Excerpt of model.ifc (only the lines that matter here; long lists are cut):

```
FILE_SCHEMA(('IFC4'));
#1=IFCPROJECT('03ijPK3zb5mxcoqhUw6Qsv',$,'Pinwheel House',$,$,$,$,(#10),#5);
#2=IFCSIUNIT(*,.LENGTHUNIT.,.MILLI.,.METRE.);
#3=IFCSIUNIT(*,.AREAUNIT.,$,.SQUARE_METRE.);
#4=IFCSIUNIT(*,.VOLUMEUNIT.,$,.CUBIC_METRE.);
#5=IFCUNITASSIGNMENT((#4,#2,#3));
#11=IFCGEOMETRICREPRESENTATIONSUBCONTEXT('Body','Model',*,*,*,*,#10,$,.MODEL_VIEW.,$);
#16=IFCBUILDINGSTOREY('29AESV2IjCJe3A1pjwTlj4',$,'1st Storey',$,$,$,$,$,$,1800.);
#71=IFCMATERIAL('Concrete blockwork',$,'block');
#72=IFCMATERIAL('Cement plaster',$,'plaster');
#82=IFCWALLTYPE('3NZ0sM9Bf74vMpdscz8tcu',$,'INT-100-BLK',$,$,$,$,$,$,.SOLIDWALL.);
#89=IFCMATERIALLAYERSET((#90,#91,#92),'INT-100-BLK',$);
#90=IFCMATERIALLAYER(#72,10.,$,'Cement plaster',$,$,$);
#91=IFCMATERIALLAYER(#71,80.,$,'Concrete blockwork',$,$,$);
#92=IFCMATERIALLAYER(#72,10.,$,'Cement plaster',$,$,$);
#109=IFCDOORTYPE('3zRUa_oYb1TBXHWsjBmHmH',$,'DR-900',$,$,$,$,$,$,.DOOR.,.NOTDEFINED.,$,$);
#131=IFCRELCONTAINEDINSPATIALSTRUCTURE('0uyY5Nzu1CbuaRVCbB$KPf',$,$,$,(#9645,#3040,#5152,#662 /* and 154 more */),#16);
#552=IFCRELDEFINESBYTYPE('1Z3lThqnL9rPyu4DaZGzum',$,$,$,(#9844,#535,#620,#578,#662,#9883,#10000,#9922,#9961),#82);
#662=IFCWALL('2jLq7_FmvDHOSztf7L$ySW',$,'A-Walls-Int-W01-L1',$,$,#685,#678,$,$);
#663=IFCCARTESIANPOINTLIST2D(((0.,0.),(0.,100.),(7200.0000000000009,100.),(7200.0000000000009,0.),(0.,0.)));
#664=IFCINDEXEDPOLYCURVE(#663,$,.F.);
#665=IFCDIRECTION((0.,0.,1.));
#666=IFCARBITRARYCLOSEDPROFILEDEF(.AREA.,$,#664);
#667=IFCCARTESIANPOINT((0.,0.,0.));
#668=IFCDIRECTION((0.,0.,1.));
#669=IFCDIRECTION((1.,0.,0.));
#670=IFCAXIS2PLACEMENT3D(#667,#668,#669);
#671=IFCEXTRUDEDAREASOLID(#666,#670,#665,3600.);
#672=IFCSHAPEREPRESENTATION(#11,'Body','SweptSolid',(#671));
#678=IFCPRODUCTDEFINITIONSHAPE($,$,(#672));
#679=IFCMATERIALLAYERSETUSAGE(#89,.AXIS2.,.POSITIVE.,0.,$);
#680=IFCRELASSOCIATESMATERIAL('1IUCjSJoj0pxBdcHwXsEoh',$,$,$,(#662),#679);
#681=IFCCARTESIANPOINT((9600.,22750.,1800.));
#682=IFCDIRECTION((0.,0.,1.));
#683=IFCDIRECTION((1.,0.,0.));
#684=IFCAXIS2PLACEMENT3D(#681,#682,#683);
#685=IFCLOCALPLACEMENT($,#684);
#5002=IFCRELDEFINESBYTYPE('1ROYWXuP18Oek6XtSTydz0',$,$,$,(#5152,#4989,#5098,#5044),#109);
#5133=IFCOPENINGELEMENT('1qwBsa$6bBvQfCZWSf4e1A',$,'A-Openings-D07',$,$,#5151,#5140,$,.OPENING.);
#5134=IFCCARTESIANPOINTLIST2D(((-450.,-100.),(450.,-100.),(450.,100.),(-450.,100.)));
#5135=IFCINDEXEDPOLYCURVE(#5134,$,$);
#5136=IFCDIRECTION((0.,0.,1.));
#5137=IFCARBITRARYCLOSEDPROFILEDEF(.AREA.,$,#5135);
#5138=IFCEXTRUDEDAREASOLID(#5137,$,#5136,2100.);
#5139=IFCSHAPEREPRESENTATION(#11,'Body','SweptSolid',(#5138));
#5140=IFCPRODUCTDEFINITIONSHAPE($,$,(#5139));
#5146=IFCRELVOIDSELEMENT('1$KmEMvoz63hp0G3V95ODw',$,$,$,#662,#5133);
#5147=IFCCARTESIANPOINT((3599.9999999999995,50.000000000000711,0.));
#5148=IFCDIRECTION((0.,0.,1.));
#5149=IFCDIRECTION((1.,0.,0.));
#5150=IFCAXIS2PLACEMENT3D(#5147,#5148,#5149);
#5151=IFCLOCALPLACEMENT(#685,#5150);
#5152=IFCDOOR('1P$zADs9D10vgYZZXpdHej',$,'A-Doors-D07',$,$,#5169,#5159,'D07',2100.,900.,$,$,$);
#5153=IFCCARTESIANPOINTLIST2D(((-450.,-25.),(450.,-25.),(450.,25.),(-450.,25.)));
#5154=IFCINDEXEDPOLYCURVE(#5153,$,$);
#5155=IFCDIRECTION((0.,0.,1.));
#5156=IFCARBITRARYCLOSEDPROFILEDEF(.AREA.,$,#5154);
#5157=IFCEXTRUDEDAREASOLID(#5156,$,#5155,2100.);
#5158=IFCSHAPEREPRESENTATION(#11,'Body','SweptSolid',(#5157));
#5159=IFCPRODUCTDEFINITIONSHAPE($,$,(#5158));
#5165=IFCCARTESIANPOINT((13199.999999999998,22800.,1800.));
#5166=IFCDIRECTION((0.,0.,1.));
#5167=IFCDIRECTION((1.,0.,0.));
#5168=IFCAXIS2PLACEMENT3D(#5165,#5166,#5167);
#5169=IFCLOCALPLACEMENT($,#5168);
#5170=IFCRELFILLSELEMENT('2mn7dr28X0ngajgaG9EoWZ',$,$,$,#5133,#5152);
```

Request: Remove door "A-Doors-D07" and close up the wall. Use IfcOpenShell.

```python
import ifcopenshell
import ifcopenshell.api.feature
import ifcopenshell.api.root
import ifcopenshell.geom
import ifcopenshell.util.shape

model = ifcopenshell.open("model.ifc")
settings = ifcopenshell.geom.settings()


def volume(element):
    """Net volume in cubic metres, openings subtracted."""
    shape = ifcopenshell.geom.create_shape(settings, element)
    return ifcopenshell.util.shape.get_volume(shape.geometry)


door = model.by_guid("1P$zADs9D10vgYZZXpdHej")
opening = door.FillsVoids[0].RelatingOpeningElement
wall = opening.VoidsElements[0].RelatingBuildingElement
before = volume(wall)

ifcopenshell.api.root.remove_product(model, product=door)
ifcopenshell.api.feature.remove_feature(model, feature=opening)

after = volume(wall)

print(f"wall volume {before:.3f} -> {after:.3f} m3")

model.write("model_updated.ifc")
```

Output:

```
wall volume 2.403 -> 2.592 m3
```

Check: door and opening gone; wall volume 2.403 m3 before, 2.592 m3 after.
